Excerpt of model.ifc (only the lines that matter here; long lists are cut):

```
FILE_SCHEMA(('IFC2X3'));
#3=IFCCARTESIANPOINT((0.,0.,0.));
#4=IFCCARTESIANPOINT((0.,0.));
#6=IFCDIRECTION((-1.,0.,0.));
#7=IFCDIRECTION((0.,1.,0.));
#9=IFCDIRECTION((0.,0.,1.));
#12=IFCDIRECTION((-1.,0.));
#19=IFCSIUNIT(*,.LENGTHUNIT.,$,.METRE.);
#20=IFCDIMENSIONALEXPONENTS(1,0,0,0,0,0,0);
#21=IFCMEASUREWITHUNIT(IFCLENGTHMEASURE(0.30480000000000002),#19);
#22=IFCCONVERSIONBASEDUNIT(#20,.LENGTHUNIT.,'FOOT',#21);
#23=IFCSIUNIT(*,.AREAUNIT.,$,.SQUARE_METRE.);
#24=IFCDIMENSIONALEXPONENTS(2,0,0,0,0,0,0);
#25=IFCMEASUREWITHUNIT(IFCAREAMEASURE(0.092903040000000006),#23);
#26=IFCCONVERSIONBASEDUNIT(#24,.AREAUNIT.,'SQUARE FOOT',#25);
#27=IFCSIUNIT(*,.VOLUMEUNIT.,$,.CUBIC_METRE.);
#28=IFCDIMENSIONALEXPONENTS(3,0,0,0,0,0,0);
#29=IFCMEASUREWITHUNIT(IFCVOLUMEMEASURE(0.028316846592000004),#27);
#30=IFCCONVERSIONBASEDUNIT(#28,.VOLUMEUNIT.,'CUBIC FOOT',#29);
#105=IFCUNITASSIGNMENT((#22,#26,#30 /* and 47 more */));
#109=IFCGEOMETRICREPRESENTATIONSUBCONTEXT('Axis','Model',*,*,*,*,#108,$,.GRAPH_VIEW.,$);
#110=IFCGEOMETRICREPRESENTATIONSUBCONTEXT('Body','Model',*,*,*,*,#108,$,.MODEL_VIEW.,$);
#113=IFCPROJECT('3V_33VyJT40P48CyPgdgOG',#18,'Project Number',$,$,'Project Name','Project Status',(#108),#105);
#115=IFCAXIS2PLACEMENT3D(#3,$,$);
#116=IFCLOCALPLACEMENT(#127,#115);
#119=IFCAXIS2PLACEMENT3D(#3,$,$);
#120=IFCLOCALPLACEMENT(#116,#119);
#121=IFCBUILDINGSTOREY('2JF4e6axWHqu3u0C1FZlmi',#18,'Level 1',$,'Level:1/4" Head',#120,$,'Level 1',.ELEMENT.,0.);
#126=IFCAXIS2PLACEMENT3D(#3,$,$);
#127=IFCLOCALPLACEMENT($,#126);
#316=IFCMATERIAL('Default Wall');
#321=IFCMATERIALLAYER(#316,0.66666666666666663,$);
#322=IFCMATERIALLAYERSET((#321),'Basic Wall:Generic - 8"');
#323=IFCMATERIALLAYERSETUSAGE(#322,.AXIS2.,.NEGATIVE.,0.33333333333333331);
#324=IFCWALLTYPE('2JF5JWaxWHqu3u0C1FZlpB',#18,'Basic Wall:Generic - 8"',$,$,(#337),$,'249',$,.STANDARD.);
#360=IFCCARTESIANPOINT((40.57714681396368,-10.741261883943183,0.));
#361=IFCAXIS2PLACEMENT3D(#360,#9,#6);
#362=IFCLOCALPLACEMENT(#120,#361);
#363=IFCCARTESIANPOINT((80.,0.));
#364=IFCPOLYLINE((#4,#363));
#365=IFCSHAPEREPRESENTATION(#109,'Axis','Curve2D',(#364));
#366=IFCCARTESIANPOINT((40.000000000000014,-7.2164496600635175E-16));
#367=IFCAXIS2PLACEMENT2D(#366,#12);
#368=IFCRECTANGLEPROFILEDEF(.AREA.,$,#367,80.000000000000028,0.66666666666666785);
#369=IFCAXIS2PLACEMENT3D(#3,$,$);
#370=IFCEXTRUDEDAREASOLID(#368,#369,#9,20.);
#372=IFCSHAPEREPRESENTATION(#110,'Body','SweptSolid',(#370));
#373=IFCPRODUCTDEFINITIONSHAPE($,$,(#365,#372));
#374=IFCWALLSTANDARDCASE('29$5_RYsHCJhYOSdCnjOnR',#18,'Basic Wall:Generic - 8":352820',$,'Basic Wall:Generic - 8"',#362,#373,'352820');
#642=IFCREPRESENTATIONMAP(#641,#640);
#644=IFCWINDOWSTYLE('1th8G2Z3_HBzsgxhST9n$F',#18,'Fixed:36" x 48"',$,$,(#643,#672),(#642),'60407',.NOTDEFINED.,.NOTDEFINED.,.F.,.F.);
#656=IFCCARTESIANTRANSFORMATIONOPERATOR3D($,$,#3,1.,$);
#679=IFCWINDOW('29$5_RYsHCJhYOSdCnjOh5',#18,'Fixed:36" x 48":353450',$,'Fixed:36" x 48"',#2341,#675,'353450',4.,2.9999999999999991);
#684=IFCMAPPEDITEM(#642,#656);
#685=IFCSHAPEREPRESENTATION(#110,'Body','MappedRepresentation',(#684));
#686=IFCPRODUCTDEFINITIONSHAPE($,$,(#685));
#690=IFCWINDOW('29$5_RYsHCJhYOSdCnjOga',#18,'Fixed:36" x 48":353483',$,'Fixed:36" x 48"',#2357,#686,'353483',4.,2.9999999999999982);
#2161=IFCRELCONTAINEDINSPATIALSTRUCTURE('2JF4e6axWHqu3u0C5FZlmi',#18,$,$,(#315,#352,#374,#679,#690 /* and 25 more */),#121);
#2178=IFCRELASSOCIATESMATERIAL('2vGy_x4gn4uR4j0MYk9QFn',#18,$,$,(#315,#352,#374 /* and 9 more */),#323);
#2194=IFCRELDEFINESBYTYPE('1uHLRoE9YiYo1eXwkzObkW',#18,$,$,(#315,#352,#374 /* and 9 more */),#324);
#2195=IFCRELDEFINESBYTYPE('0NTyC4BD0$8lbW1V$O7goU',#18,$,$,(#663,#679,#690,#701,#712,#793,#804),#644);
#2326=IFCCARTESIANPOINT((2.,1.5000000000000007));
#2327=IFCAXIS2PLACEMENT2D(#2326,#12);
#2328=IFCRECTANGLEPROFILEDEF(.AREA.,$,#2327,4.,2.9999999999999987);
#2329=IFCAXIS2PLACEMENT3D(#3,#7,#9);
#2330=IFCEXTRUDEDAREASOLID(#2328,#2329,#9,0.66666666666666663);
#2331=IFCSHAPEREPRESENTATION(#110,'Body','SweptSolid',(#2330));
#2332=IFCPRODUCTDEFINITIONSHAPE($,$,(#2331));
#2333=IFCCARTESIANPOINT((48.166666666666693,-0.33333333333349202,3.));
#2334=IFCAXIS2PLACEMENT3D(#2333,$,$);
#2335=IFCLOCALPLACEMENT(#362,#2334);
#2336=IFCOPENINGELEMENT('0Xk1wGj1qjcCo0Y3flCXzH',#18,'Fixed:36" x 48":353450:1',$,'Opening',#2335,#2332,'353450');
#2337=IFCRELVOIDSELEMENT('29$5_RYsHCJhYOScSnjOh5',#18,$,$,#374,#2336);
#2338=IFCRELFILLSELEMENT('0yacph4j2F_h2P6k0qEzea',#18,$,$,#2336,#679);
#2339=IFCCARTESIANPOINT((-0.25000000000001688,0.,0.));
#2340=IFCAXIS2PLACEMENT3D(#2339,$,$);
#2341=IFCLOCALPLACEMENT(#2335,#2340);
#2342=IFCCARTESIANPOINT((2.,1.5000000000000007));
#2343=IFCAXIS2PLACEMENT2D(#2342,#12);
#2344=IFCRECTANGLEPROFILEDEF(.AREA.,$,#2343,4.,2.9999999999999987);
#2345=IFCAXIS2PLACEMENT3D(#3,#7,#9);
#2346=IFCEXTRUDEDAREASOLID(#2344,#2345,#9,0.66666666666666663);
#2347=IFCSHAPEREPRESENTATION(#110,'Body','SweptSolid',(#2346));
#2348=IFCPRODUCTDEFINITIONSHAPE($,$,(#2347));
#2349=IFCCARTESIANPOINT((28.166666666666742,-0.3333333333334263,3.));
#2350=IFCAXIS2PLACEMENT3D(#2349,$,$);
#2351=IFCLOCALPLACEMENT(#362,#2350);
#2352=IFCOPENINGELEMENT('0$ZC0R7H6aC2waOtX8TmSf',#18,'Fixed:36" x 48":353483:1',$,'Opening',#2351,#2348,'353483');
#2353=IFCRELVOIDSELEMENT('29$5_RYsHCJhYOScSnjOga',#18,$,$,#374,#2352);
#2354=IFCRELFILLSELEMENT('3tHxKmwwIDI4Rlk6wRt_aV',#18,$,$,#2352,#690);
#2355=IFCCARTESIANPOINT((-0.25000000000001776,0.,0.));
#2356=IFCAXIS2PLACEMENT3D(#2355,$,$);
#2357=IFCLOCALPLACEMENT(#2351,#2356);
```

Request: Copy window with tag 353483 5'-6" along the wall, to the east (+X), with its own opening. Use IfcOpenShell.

```python
import ifcopenshell
import ifcopenshell.api.feature
import ifcopenshell.api.geometry
import ifcopenshell.api.root
import ifcopenshell.geom
import ifcopenshell.util.element
import ifcopenshell.util.placement
import ifcopenshell.util.shape
import ifcopenshell.util.unit

model = ifcopenshell.open("model.ifc")
unit_scale = ifcopenshell.util.unit.calculate_unit_scale(model)
settings = ifcopenshell.geom.settings()


def volume(element):
    """Net volume in cubic metres, openings subtracted."""
    shape = ifcopenshell.geom.create_shape(settings, element)
    return ifcopenshell.util.shape.get_volume(shape.geometry)


def reuse_history(source, copy):
    """copy_class also copies each property set's owner history, people and application; keep the originals."""
    for rel in copy.IsDefinedBy:
        if rel.is_a("IfcRelDefinesByProperties") and (history := rel.RelatingPropertyDefinition.OwnerHistory):
            rel.RelatingPropertyDefinition.OwnerHistory = source.OwnerHistory
            ifcopenshell.util.element.remove_deep2(model, history)


window = model.by_guid("29$5_RYsHCJhYOSdCnjOga")
opening = window.FillsVoids[0].RelatingOpeningElement
wall = opening.VoidsElements[0].RelatingBuildingElement
before = volume(wall)
shift = ifcopenshell.util.placement.get_local_placement(wall.ObjectPlacement)[:3, 0] * -66 * 0.0254 / unit_scale

# copy_class copies the void relationship, type, container and properties, but no geometry.
new_opening = ifcopenshell.api.root.copy_class(model, product=opening)
new_opening.Representation = ifcopenshell.util.element.copy_deep(
    model, opening.Representation, exclude=["IfcGeometricRepresentationContext", "IfcRepresentationMap"]
)
new_opening.Name = 'Fixed:36" x 48"'
new_opening.Tag = None
new_window = ifcopenshell.api.root.copy_class(model, product=window)
new_window.Representation = ifcopenshell.util.element.copy_deep(
    model, window.Representation, exclude=["IfcGeometricRepresentationContext", "IfcRepresentationMap"]
)
new_window.Name = 'Fixed:36" x 48"'
new_window.Tag = None
reuse_history(window, new_window)
fills = ifcopenshell.api.feature.add_filling(model, opening=new_opening, element=new_window)
fills.OwnerHistory = new_window.OwnerHistory  # required in IFC2X3

for old, new in ((opening, new_opening), (window, new_window)):
    matrix = ifcopenshell.util.placement.get_local_placement(old.ObjectPlacement)
    matrix[:3, 3] += shift
    ifcopenshell.api.geometry.edit_object_placement(model, product=new, matrix=matrix, is_si=False)

after = volume(wall)

print(f"wall volume {before:.3f} -> {after:.3f} m3")

model.write("model_rev.ifc")
```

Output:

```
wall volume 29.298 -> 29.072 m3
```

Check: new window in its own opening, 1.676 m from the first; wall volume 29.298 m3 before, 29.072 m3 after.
